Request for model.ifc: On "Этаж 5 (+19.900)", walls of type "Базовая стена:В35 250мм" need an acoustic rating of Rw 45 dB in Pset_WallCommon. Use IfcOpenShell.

First a look at what the model holds.

```python
import ifcopenshell
import ifcopenshell.util.element

model = ifcopenshell.open("model.ifc")
print(model.schema)
storey = next(s for s in model.by_type("IfcBuildingStorey") if s.Name == "Этаж 5 (+19.900)")
walls = [e for e in ifcopenshell.util.element.get_decomposition(storey) if e.is_a("IfcWall")]
seen = {}
for e in walls:
    element_type = ifcopenshell.util.element.get_type(e)
    key = (element_type.Name if element_type != e and element_type else None, ifcopenshell.util.element.get_pset(e, "Pset_WallCommon", "AcousticRating"))
    seen[key] = seen.get(key, 0) + 1
for (name, value), count in sorted(seen.items(), key=str):
    print(count, "x", name, "|", value)
```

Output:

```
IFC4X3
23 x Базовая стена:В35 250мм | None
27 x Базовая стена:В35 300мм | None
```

```python
import ifcopenshell
import ifcopenshell.api.pset
import ifcopenshell.util.element

model = ifcopenshell.open("model.ifc")

storey = next(s for s in model.by_type("IfcBuildingStorey") if s.Name == "Этаж 5 (+19.900)")
walls = [e for e in ifcopenshell.util.element.get_decomposition(storey) if e.is_a("IfcWall")]

count = 0
for e in walls:
    element_type = ifcopenshell.util.element.get_type(e)
    if element_type in (None, e) or element_type.Name != "Базовая стена:В35 250мм":
        continue
    # add_pset returns the element's existing set when there is one.
    pset = ifcopenshell.api.pset.add_pset(model, product=e, name="Pset_WallCommon")
    ifcopenshell.api.pset.edit_pset(model, pset=pset, properties={"AcousticRating": "Rw 45 dB"})
    count += 1

print(count, "walls updated")

model.write("model_v2.ifc")
```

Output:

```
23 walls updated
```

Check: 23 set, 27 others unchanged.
